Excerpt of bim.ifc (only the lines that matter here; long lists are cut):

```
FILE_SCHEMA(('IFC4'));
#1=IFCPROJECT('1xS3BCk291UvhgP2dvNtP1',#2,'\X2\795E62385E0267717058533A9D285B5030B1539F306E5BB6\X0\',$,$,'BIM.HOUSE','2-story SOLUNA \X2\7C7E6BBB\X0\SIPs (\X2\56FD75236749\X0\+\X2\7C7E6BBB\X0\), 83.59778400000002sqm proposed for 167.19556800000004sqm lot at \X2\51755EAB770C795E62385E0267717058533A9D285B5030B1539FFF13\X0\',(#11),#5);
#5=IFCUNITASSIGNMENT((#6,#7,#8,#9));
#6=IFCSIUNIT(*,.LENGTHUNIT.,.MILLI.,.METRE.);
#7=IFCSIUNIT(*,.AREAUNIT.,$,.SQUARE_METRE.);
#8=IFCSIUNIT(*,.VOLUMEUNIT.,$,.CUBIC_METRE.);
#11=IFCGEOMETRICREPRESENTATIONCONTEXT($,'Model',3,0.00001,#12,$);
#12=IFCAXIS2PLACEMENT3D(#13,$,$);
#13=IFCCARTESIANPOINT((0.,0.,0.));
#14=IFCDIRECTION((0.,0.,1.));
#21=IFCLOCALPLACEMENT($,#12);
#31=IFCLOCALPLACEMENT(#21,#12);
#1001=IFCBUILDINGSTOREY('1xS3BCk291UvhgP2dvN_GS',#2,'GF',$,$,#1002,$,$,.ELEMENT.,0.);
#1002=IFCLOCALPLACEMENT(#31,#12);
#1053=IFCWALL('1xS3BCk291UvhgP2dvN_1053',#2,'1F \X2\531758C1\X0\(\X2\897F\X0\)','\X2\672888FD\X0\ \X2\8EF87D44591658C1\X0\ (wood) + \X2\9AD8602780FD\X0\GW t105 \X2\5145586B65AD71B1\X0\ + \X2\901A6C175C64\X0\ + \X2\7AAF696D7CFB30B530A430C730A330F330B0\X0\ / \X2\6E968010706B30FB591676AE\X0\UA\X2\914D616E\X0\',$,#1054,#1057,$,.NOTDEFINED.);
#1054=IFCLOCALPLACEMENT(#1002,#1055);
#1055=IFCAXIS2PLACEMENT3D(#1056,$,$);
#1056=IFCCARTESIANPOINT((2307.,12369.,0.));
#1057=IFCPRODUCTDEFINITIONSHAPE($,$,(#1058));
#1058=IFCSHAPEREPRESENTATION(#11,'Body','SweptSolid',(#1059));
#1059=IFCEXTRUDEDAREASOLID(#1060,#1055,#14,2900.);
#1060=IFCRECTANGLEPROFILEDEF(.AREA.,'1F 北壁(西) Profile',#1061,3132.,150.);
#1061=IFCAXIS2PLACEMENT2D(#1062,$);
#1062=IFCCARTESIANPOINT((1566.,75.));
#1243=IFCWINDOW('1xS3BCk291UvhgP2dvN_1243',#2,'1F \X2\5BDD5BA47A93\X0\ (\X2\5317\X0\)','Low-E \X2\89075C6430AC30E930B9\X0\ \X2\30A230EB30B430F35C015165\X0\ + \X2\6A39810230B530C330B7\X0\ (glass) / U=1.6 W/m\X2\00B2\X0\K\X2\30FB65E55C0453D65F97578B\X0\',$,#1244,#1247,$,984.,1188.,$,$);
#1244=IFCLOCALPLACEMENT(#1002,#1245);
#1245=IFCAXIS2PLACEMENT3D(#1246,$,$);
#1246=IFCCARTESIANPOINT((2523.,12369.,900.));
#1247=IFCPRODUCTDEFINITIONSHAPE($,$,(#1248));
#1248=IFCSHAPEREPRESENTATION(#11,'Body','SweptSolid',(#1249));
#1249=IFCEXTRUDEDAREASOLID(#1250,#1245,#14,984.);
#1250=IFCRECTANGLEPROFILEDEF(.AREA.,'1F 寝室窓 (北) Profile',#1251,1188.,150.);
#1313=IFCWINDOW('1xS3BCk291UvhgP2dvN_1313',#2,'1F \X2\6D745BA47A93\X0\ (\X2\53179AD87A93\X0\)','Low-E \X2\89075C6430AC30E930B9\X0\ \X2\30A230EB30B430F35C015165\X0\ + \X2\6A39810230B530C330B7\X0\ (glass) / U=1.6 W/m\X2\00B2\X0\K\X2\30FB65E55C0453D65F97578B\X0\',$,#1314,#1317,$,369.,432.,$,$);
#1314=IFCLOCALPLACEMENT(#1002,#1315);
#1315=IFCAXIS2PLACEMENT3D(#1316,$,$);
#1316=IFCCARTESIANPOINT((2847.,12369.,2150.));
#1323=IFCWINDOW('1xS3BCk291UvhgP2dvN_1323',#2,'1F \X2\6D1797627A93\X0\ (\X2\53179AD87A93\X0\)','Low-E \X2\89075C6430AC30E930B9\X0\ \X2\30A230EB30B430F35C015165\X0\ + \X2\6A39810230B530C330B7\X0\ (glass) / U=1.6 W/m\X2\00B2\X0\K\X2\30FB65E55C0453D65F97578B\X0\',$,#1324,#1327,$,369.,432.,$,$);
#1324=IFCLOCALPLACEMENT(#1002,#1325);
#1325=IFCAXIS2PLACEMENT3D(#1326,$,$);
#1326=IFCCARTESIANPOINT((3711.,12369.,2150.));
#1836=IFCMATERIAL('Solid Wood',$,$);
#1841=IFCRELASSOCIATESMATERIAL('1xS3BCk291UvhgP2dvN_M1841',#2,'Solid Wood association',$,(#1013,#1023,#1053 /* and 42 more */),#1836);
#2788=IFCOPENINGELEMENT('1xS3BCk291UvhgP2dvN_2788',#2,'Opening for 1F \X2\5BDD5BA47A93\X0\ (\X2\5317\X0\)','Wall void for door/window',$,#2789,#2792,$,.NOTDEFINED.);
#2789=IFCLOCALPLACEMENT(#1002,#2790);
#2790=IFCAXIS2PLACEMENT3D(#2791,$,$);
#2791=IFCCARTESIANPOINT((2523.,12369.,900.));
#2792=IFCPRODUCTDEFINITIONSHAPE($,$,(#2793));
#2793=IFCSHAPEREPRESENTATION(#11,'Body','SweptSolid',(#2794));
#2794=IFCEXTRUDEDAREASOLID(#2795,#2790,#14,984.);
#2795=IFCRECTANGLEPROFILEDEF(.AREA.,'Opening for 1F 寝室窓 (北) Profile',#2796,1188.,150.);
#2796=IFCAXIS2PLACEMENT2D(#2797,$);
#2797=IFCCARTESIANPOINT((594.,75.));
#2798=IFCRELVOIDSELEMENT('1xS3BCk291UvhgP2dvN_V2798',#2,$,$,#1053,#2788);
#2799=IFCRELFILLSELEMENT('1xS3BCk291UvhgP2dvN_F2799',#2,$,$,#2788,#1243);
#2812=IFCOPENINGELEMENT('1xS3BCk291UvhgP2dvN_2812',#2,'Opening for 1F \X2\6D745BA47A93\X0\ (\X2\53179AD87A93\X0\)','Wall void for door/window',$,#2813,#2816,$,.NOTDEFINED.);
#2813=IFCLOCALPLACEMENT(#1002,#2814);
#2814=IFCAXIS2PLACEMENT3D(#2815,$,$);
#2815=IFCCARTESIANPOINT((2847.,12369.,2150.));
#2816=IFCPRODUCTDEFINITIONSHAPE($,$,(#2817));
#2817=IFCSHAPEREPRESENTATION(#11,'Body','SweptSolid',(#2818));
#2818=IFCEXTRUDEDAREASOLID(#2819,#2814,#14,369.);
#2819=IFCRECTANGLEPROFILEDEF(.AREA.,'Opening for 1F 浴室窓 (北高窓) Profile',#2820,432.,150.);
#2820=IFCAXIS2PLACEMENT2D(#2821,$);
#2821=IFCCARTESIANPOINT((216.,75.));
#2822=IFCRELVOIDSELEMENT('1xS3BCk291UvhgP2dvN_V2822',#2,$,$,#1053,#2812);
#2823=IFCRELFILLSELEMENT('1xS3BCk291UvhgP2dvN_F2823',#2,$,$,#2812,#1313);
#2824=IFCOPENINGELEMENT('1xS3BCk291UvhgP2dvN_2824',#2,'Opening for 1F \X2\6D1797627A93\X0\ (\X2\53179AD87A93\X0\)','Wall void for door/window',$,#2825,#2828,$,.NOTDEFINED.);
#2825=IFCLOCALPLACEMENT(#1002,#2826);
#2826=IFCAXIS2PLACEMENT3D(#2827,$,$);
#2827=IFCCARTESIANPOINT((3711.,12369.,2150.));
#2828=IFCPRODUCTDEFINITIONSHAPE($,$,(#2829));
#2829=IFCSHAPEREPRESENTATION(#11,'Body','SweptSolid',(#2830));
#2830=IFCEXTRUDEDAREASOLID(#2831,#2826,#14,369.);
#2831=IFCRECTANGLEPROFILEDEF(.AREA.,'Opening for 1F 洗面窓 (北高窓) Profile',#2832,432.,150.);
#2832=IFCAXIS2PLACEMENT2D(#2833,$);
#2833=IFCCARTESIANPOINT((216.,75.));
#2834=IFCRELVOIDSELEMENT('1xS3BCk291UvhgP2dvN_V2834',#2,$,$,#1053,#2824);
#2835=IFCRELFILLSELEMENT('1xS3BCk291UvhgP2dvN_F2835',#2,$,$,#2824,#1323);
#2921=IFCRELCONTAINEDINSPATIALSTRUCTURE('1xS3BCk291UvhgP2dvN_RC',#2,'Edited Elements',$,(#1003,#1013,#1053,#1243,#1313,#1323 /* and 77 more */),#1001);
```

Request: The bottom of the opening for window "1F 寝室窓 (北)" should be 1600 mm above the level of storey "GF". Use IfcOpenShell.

```python
import numpy as np
import ifcopenshell
import ifcopenshell.api.geometry
import ifcopenshell.geom
import ifcopenshell.util.element
import ifcopenshell.util.placement
import ifcopenshell.util.shape
import ifcopenshell.util.unit

model = ifcopenshell.open("bim.ifc")
unit_scale = ifcopenshell.util.unit.calculate_unit_scale(model)

window = model.by_guid("1xS3BCk291UvhgP2dvN_1243")
opening = window.FillsVoids[0].RelatingOpeningElement
storey = ifcopenshell.util.element.get_container(window, ifc_class="IfcBuildingStorey")
level = ifcopenshell.util.placement.get_local_placement(storey.ObjectPlacement)[2, 3]

# The opening's origin need not be at the sill, so measure its lowest point.
shape = ifcopenshell.geom.create_shape(ifcopenshell.geom.settings(), opening)
bottom = ifcopenshell.util.shape.get_shape_bottom_elevation(shape, shape.geometry) / unit_scale
dz = level + 1.6 / unit_scale - bottom

shift = np.array([0.0, 0.0, dz])
# The window is not placed relative to its opening, so move both.
for product in (opening, window):
    matrix = ifcopenshell.util.placement.get_local_placement(product.ObjectPlacement)
    matrix[:3, 3] += shift
    ifcopenshell.api.geometry.edit_object_placement(model, product=product, matrix=matrix, is_si=False)

print(f"moved by {dz * unit_scale:+.3f} m")

model.write("bim_updated.ifc")
```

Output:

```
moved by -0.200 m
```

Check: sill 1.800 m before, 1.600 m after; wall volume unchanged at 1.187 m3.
